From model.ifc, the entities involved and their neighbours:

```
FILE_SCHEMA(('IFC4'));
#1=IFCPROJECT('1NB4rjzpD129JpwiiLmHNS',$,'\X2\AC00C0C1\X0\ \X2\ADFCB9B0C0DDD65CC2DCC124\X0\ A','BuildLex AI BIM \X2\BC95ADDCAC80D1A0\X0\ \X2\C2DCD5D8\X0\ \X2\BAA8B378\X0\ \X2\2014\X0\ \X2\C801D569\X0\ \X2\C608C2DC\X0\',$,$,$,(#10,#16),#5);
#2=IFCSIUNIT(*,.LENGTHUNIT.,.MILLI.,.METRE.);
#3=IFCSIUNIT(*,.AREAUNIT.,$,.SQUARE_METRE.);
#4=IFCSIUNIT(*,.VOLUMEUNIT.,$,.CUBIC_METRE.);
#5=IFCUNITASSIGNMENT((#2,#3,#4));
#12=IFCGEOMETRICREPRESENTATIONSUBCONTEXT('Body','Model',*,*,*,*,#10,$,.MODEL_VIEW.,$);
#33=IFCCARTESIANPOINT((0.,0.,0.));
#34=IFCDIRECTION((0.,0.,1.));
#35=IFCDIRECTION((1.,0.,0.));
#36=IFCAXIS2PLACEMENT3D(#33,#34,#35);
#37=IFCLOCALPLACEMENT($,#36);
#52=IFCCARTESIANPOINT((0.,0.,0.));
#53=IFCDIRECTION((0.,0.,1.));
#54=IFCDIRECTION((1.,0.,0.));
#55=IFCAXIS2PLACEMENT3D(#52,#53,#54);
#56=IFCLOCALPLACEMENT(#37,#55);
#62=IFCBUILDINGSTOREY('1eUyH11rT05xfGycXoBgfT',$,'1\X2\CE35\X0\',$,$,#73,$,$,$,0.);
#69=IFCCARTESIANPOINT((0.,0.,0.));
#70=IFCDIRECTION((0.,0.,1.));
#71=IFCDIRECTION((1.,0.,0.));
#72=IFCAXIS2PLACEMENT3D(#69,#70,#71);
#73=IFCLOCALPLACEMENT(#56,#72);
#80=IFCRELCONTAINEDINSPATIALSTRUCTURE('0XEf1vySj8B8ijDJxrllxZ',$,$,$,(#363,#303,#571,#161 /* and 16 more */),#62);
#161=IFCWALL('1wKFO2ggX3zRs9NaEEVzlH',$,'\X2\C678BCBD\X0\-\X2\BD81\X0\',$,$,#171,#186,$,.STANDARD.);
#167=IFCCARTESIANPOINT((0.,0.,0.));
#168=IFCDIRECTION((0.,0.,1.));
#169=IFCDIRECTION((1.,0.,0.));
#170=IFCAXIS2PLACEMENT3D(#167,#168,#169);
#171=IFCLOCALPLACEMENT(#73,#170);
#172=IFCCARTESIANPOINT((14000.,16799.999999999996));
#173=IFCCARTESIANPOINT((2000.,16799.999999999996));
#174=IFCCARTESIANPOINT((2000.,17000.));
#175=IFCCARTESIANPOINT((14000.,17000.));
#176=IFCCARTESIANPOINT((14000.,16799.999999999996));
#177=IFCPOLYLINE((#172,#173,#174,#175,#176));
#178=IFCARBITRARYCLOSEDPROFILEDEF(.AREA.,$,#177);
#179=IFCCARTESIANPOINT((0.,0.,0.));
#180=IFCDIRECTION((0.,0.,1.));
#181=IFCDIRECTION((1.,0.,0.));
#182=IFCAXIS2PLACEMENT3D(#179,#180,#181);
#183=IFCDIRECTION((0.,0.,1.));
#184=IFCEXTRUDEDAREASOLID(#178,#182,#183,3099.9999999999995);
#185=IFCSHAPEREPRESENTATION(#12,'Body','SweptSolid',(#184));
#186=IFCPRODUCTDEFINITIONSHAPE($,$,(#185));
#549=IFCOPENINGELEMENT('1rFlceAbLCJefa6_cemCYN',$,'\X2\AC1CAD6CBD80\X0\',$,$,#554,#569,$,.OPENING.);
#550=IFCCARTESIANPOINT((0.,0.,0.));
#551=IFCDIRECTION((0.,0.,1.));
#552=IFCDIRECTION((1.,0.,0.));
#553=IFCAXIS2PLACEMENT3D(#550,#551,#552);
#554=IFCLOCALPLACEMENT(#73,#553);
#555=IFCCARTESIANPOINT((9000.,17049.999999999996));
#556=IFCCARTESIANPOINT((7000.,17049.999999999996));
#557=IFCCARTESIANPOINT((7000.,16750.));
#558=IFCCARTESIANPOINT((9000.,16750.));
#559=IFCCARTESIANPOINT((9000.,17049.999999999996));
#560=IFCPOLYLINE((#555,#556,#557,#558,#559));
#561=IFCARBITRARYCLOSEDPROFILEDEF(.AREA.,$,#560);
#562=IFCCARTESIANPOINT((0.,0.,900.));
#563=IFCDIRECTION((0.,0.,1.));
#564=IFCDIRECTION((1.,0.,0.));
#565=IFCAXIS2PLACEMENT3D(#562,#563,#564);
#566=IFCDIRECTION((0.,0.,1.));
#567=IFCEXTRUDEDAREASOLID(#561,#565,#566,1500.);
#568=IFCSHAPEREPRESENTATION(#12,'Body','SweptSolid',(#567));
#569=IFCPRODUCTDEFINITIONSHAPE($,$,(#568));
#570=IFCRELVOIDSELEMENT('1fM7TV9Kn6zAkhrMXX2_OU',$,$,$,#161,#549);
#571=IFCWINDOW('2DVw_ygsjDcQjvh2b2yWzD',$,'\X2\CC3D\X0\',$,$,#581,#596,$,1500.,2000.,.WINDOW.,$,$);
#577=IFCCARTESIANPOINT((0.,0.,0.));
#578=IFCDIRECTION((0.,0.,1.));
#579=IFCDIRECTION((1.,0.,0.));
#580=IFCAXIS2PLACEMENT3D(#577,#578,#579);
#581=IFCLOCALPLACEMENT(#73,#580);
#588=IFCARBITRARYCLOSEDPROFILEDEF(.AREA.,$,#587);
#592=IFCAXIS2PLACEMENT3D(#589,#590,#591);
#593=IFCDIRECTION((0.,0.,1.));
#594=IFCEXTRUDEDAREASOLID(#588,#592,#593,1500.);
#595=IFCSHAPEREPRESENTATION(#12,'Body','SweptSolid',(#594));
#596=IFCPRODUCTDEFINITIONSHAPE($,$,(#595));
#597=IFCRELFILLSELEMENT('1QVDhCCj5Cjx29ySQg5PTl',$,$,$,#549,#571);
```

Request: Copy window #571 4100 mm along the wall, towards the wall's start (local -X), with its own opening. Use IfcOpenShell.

```python
import ifcopenshell
import ifcopenshell.api.feature
import ifcopenshell.api.geometry
import ifcopenshell.api.root
import ifcopenshell.geom
import ifcopenshell.util.element
import ifcopenshell.util.placement
import ifcopenshell.util.shape
import ifcopenshell.util.unit

model = ifcopenshell.open("model.ifc")
unit_scale = ifcopenshell.util.unit.calculate_unit_scale(model)
settings = ifcopenshell.geom.settings()


def volume(element):
    """Net volume in cubic metres, openings subtracted."""
    shape = ifcopenshell.geom.create_shape(settings, element)
    return ifcopenshell.util.shape.get_volume(shape.geometry)


window = model.by_guid("2DVw_ygsjDcQjvh2b2yWzD")
opening = window.FillsVoids[0].RelatingOpeningElement
wall = opening.VoidsElements[0].RelatingBuildingElement
before = volume(wall)
shift = ifcopenshell.util.placement.get_local_placement(wall.ObjectPlacement)[:3, 0] * -4.1 / unit_scale

# copy_class copies the void relationship, type, container and properties, but no geometry.
new_opening = ifcopenshell.api.root.copy_class(model, product=opening)
new_opening.Representation = ifcopenshell.util.element.copy_deep(
    model, opening.Representation, exclude=["IfcGeometricRepresentationContext", "IfcRepresentationMap"]
)
new_window = ifcopenshell.api.root.copy_class(model, product=window)
new_window.Representation = ifcopenshell.util.element.copy_deep(
    model, window.Representation, exclude=["IfcGeometricRepresentationContext", "IfcRepresentationMap"]
)
ifcopenshell.api.feature.add_filling(model, opening=new_opening, element=new_window)

for old, new in ((opening, new_opening), (window, new_window)):
    matrix = ifcopenshell.util.placement.get_local_placement(old.ObjectPlacement)
    matrix[:3, 3] += shift
    ifcopenshell.api.geometry.edit_object_placement(model, product=new, matrix=matrix, is_si=False)

after = volume(wall)

print(f"wall volume {before:.3f} -> {after:.3f} m3")

model.write("model-out.ifc")
```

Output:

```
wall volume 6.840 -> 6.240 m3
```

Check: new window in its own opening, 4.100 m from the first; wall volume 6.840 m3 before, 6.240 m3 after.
